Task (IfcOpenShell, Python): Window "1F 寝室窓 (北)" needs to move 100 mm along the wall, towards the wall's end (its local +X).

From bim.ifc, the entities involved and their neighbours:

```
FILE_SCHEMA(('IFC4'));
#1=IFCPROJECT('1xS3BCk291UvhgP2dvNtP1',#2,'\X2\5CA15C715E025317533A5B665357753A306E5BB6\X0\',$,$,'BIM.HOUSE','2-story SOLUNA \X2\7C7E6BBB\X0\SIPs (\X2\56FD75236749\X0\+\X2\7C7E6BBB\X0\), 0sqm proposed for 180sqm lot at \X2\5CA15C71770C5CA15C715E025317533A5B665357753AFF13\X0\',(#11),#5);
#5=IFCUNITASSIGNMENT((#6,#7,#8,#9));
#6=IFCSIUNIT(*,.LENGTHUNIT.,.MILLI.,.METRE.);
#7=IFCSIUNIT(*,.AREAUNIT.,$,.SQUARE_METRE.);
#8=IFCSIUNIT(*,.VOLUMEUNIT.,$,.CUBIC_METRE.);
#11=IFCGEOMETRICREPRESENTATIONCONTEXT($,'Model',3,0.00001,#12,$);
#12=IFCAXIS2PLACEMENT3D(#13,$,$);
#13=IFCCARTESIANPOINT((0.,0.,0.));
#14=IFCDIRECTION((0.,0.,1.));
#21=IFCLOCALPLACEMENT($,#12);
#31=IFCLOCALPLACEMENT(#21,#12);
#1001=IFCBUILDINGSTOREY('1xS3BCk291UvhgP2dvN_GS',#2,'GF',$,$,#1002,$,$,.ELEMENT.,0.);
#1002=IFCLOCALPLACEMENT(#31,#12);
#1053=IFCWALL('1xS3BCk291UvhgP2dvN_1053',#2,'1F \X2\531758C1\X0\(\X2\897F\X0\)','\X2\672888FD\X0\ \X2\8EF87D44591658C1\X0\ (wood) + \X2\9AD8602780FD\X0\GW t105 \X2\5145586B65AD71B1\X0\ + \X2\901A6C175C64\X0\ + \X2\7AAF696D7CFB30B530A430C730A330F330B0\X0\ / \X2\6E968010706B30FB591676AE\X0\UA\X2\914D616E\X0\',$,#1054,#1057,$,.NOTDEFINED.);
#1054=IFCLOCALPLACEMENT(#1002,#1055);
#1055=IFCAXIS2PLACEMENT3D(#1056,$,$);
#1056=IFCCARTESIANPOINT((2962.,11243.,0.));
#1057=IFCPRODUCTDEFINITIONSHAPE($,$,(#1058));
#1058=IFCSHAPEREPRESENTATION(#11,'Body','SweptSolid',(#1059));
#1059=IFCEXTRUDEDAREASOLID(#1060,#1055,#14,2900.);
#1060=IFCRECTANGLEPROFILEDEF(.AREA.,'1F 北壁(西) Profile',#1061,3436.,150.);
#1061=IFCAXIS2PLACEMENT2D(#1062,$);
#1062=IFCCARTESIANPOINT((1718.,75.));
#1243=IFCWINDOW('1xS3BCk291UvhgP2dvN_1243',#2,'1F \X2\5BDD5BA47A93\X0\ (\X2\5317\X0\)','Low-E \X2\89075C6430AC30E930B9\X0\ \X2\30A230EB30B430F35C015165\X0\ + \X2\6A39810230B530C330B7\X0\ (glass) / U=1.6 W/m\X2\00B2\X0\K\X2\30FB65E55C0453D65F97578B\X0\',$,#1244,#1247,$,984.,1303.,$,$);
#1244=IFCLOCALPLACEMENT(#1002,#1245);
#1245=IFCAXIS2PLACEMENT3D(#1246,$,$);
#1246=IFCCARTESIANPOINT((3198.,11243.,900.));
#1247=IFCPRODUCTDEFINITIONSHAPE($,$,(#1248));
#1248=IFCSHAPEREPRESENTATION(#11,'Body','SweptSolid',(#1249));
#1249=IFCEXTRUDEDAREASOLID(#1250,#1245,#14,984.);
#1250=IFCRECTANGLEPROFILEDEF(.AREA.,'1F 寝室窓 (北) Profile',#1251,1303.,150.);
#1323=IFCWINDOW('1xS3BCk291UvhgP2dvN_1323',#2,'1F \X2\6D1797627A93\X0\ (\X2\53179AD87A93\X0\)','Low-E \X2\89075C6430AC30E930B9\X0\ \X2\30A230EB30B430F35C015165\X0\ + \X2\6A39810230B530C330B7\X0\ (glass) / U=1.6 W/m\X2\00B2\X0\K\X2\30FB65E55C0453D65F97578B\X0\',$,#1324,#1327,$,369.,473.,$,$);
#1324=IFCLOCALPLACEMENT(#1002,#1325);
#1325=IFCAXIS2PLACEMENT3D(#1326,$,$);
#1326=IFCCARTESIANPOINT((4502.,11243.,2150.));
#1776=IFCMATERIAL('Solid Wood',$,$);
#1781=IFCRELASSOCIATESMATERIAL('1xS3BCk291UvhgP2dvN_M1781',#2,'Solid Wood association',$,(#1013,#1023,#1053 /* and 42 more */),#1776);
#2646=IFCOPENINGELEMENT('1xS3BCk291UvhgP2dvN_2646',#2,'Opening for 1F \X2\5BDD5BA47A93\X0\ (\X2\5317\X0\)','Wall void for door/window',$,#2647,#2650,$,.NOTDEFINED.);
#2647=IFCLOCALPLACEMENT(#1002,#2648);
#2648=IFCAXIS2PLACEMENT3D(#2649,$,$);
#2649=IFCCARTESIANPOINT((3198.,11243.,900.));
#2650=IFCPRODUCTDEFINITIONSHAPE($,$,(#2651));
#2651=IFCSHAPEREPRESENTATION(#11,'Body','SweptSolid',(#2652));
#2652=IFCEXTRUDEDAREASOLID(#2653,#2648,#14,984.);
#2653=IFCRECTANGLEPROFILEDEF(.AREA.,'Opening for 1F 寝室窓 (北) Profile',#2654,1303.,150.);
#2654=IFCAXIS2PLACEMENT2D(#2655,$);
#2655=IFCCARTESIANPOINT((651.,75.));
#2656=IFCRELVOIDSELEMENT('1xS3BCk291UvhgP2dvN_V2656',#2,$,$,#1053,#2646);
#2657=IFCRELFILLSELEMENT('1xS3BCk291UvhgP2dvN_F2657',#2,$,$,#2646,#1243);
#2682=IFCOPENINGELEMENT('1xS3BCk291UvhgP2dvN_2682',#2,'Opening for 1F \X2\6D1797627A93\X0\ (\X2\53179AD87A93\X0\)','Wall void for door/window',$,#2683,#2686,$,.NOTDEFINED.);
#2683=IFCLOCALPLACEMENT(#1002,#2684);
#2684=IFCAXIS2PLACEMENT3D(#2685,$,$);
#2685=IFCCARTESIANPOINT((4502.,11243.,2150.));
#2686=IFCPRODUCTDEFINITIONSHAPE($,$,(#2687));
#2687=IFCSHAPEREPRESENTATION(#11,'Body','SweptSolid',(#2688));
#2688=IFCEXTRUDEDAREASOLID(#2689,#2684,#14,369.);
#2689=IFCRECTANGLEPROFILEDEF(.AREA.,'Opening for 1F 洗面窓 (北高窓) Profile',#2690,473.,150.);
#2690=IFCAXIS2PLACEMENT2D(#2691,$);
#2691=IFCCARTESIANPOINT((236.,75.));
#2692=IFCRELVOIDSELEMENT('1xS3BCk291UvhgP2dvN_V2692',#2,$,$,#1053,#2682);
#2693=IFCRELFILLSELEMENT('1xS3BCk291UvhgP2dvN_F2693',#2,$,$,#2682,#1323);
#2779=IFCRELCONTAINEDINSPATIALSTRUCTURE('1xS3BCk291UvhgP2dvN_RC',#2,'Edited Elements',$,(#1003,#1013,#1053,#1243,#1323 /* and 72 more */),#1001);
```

```python
import ifcopenshell
import ifcopenshell.api.geometry
import ifcopenshell.util.placement

model = ifcopenshell.open("bim.ifc")

window = model.by_guid("1xS3BCk291UvhgP2dvN_1243")
opening = window.FillsVoids[0].RelatingOpeningElement
wall = opening.VoidsElements[0].RelatingBuildingElement

wall_matrix = ifcopenshell.util.placement.get_local_placement(wall.ObjectPlacement)
shift = wall_matrix[:3, 0] * 100.0
before = ifcopenshell.util.placement.get_local_placement(window.ObjectPlacement)[:3, 3].copy()

# The window is not placed relative to its opening, so move both.
for product in (opening, window):
    matrix = ifcopenshell.util.placement.get_local_placement(product.ObjectPlacement)
    matrix[:3, 3] += shift
    ifcopenshell.api.geometry.edit_object_placement(model, product=product, matrix=matrix, is_si=False)

after = ifcopenshell.util.placement.get_local_placement(window.ObjectPlacement)[:3, 3]
print("window moved by", (after - before).round(3) + 0.0)

model.write("bim-out.ifc")
```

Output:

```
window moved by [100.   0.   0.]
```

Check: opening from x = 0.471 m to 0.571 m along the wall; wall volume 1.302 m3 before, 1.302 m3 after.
